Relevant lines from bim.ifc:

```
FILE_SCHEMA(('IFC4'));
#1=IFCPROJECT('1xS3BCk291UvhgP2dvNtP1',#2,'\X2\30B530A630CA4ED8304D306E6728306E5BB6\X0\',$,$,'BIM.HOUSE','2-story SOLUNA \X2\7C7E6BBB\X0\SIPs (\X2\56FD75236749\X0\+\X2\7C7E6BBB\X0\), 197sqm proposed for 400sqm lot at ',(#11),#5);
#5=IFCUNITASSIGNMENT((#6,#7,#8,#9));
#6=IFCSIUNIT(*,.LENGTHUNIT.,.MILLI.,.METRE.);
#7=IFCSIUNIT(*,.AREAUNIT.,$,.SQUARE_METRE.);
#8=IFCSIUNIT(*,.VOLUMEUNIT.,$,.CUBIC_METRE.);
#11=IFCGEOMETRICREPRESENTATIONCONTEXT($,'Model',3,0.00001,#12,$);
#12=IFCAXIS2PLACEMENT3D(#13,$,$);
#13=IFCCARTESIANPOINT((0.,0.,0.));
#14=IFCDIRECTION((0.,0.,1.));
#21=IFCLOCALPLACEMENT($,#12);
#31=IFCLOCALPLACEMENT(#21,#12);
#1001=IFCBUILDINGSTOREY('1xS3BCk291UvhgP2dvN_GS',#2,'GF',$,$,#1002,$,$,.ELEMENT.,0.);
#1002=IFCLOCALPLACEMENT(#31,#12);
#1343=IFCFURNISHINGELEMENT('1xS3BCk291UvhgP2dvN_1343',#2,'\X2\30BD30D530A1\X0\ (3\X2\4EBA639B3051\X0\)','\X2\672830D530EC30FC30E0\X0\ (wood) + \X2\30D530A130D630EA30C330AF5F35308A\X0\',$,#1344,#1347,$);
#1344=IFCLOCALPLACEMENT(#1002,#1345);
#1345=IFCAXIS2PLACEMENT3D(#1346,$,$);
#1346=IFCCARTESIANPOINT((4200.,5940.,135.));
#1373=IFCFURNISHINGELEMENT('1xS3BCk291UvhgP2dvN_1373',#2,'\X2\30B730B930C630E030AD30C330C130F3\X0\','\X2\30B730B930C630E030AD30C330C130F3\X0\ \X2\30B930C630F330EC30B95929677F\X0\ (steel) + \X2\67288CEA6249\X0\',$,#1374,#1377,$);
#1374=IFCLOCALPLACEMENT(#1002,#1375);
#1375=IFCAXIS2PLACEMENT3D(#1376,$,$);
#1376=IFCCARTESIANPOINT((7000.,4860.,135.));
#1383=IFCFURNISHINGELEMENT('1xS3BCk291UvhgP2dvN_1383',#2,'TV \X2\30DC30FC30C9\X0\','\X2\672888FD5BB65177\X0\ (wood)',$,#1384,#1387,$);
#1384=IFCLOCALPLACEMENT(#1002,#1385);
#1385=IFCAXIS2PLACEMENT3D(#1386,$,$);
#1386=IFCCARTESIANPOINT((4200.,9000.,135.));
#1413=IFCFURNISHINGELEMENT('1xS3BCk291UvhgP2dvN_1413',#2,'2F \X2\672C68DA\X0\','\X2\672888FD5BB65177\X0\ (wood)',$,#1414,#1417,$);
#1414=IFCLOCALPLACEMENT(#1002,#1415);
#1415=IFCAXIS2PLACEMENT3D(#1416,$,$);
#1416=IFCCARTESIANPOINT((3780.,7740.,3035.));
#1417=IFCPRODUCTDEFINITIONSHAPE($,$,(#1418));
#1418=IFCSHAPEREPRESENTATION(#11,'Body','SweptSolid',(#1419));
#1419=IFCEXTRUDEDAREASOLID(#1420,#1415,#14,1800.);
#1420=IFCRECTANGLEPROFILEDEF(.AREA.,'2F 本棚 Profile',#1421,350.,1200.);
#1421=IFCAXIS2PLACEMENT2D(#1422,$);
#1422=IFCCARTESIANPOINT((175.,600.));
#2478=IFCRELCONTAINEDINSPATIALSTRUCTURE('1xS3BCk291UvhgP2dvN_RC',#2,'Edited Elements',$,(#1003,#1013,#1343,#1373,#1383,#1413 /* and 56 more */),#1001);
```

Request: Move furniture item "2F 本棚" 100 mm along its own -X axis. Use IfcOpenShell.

```python
import ifcopenshell
import ifcopenshell.api.geometry
import ifcopenshell.util.placement

model = ifcopenshell.open("bim.ifc")

item = model.by_guid("1xS3BCk291UvhgP2dvN_1413")
matrix = ifcopenshell.util.placement.get_local_placement(item.ObjectPlacement)
matrix[:3, 3] -= matrix[:3, 0] * 100.0
ifcopenshell.api.geometry.edit_object_placement(model, product=item, matrix=matrix, is_si=False)

print(ifcopenshell.util.placement.get_local_placement(item.ObjectPlacement).round(3) + 0.0)

model.write("bim_rev.ifc")
```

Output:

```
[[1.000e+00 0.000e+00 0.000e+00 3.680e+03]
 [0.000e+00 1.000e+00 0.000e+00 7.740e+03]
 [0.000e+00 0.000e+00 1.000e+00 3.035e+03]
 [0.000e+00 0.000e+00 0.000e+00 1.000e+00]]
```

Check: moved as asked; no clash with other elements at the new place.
